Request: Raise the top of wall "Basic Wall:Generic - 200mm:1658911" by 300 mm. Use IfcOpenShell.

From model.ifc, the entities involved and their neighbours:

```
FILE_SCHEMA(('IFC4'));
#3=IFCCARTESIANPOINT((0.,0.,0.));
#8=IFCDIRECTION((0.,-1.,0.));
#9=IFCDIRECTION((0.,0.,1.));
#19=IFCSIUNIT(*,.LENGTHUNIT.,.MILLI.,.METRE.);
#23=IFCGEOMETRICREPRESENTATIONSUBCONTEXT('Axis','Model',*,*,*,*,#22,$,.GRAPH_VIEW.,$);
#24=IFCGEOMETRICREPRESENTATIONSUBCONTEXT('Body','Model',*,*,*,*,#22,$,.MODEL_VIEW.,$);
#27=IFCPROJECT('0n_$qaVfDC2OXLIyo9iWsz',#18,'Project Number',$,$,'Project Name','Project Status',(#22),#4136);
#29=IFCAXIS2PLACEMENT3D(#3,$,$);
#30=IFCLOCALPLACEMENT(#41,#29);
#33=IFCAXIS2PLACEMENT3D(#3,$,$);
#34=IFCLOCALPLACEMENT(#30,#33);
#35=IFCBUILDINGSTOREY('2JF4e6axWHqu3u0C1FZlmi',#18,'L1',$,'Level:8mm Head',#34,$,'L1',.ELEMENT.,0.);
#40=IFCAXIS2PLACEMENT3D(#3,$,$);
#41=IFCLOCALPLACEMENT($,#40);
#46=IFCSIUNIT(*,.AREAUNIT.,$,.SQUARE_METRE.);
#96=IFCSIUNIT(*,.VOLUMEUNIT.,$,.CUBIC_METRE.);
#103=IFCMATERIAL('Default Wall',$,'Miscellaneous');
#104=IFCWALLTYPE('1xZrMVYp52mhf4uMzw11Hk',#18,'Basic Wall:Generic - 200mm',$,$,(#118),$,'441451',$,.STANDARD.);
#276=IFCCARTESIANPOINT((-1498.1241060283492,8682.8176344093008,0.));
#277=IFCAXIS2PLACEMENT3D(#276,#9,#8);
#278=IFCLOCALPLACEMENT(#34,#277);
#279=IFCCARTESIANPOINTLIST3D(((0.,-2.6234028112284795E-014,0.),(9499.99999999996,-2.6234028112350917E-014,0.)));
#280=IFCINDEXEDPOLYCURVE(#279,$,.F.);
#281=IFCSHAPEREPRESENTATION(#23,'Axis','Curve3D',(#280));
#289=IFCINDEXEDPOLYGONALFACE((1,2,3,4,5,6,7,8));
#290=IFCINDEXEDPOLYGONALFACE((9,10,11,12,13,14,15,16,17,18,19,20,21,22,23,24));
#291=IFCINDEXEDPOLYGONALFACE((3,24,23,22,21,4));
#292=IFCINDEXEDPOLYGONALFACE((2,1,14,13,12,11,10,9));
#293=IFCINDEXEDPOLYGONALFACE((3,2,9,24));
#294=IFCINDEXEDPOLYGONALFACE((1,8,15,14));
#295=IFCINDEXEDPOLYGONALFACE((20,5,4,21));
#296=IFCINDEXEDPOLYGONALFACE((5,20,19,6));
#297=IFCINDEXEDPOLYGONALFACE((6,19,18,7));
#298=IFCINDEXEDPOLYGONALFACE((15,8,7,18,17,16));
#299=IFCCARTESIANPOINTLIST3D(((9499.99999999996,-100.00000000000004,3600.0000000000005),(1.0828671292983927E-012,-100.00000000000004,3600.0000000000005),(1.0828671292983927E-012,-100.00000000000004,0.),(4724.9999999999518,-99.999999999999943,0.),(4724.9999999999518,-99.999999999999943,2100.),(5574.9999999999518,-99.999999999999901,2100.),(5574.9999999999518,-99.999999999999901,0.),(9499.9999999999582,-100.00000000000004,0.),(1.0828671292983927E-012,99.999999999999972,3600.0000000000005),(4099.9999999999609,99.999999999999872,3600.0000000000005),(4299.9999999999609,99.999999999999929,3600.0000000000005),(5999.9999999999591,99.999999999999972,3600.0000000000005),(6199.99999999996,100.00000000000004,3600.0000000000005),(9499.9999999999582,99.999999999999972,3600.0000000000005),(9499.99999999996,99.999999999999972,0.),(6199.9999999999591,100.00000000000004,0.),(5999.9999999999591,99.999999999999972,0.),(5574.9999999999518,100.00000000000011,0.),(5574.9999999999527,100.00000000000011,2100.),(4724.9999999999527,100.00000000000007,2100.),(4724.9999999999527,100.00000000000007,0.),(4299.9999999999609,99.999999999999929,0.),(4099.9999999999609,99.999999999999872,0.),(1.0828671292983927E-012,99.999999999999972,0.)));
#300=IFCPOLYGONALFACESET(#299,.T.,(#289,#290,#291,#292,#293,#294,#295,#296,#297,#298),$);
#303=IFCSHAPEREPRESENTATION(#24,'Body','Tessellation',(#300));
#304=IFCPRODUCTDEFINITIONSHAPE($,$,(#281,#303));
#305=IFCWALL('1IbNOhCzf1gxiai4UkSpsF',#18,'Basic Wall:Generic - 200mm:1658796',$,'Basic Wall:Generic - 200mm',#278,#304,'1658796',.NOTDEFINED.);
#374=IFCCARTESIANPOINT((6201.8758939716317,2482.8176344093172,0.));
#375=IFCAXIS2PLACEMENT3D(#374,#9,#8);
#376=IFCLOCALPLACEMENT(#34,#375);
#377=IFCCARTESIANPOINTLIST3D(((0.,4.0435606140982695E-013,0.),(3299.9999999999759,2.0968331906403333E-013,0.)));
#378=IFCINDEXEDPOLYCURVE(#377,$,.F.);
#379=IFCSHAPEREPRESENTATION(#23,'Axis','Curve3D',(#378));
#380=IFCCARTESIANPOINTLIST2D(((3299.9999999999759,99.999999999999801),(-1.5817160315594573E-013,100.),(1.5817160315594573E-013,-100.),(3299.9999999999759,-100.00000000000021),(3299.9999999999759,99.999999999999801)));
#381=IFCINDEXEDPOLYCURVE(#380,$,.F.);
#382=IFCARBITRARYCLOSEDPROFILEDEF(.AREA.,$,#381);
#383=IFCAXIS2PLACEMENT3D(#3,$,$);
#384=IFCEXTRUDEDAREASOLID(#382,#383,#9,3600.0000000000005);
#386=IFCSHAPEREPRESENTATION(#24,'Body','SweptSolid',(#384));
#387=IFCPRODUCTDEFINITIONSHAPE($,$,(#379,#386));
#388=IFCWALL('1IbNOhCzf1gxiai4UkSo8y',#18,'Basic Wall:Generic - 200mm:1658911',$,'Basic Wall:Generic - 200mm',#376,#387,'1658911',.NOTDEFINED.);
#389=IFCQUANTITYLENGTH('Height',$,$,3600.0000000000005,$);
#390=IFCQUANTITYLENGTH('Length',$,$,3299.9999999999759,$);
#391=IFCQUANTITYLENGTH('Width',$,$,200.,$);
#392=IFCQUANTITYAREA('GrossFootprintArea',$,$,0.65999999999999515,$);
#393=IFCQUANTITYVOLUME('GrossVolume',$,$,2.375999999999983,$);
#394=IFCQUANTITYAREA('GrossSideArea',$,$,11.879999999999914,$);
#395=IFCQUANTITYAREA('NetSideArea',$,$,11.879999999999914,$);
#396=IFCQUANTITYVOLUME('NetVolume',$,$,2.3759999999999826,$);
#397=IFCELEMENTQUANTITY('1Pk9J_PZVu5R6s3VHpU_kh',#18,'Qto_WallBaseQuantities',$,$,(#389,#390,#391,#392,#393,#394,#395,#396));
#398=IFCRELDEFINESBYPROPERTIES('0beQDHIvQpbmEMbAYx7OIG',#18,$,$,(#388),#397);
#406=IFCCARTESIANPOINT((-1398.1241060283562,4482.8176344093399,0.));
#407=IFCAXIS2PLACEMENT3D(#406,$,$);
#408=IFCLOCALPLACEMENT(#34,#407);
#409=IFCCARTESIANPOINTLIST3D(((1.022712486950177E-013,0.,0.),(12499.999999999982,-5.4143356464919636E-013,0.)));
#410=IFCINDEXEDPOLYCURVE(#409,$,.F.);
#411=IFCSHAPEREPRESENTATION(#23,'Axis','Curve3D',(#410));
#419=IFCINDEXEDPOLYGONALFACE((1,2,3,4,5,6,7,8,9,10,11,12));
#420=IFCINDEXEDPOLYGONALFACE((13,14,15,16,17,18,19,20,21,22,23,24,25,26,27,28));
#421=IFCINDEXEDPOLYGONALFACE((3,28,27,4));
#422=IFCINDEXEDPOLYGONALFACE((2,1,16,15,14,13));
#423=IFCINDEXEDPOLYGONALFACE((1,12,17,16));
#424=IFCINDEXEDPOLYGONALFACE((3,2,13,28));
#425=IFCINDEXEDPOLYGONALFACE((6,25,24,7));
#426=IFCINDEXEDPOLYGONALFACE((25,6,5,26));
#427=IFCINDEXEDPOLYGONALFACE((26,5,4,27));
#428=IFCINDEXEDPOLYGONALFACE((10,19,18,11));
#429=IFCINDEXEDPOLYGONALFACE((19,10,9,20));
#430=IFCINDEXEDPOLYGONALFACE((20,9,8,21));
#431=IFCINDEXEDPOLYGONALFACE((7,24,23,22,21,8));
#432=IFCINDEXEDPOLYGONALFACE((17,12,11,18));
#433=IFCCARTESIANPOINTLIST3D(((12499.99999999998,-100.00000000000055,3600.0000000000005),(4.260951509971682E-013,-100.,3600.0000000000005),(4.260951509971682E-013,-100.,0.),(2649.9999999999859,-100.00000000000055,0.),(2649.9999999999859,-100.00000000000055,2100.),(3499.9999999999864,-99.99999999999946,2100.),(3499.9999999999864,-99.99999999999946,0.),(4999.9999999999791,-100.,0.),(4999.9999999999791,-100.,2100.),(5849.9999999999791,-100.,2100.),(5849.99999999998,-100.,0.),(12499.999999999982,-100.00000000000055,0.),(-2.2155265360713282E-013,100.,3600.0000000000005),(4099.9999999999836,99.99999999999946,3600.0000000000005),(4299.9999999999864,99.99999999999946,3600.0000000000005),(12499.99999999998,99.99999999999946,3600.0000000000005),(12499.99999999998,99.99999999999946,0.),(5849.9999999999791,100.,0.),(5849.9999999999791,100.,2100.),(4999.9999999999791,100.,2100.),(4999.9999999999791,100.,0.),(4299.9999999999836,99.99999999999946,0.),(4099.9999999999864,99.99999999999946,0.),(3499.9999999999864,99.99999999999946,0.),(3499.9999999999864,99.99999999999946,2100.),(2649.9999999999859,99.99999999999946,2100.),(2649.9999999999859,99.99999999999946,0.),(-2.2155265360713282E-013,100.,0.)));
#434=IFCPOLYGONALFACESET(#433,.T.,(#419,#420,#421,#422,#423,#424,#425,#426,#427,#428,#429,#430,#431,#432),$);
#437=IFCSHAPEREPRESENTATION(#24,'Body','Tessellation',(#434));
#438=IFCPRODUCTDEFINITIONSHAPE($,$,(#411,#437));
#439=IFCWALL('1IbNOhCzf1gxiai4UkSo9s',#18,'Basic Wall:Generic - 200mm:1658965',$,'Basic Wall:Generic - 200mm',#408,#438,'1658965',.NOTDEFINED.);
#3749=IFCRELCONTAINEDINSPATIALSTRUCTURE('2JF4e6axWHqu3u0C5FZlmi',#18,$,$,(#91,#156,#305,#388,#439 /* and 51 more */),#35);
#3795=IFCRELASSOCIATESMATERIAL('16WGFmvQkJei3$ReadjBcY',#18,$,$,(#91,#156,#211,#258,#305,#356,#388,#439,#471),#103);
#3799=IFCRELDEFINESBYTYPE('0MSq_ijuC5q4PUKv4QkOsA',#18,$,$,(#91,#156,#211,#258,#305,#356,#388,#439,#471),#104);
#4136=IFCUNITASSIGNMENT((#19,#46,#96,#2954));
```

```python
import ifcopenshell
import ifcopenshell.api.pset
import ifcopenshell.geom
import ifcopenshell.util.element
import ifcopenshell.util.representation
import ifcopenshell.util.shape
import ifcopenshell.util.unit

model = ifcopenshell.open("model.ifc")
unit_scale = ifcopenshell.util.unit.calculate_unit_scale(model)
area_scale = ifcopenshell.util.unit.calculate_unit_scale(model, "AREAUNIT")
volume_scale = ifcopenshell.util.unit.calculate_unit_scale(model, "VOLUMEUNIT")
settings = ifcopenshell.geom.settings()


def volume(element):
    """Net volume in cubic metres, openings subtracted."""
    shape = ifcopenshell.geom.create_shape(settings, element)
    return ifcopenshell.util.shape.get_volume(shape.geometry)


wall = model.by_guid("1IbNOhCzf1gxiai4UkSo8y")
before = volume(wall)

body = ifcopenshell.util.representation.get_representation(wall, "Model", "Body")
solid = body.Items[0]
old_height = solid.Depth
solid.Depth += 300.0
after = volume(wall)
thickness = 0.2  # wall thickness in metres

# Update the stored height, areas and volumes.
qto = model.by_id(ifcopenshell.util.element.get_pset(wall, "Qto_WallBaseQuantities", should_inherit=False)["id"])
ifcopenshell.api.pset.edit_qto(model, qto=qto, properties={
    "Height": solid.Depth,
    "GrossVolume": ifcopenshell.util.element.get_pset(wall, "Qto_WallBaseQuantities", "GrossVolume") * solid.Depth / old_height,
    "GrossSideArea": ifcopenshell.util.element.get_pset(wall, "Qto_WallBaseQuantities", "GrossSideArea") * solid.Depth / old_height,
    "NetSideArea": after / thickness / area_scale,
    "NetVolume": after / volume_scale,
})

print(f"height {old_height:g} -> {solid.Depth:g}, volume {before:.3f} -> {after:.3f} m3")

model.write("model_edited.ifc")
```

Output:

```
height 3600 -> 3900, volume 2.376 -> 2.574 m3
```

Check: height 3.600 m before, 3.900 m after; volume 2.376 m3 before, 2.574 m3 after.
